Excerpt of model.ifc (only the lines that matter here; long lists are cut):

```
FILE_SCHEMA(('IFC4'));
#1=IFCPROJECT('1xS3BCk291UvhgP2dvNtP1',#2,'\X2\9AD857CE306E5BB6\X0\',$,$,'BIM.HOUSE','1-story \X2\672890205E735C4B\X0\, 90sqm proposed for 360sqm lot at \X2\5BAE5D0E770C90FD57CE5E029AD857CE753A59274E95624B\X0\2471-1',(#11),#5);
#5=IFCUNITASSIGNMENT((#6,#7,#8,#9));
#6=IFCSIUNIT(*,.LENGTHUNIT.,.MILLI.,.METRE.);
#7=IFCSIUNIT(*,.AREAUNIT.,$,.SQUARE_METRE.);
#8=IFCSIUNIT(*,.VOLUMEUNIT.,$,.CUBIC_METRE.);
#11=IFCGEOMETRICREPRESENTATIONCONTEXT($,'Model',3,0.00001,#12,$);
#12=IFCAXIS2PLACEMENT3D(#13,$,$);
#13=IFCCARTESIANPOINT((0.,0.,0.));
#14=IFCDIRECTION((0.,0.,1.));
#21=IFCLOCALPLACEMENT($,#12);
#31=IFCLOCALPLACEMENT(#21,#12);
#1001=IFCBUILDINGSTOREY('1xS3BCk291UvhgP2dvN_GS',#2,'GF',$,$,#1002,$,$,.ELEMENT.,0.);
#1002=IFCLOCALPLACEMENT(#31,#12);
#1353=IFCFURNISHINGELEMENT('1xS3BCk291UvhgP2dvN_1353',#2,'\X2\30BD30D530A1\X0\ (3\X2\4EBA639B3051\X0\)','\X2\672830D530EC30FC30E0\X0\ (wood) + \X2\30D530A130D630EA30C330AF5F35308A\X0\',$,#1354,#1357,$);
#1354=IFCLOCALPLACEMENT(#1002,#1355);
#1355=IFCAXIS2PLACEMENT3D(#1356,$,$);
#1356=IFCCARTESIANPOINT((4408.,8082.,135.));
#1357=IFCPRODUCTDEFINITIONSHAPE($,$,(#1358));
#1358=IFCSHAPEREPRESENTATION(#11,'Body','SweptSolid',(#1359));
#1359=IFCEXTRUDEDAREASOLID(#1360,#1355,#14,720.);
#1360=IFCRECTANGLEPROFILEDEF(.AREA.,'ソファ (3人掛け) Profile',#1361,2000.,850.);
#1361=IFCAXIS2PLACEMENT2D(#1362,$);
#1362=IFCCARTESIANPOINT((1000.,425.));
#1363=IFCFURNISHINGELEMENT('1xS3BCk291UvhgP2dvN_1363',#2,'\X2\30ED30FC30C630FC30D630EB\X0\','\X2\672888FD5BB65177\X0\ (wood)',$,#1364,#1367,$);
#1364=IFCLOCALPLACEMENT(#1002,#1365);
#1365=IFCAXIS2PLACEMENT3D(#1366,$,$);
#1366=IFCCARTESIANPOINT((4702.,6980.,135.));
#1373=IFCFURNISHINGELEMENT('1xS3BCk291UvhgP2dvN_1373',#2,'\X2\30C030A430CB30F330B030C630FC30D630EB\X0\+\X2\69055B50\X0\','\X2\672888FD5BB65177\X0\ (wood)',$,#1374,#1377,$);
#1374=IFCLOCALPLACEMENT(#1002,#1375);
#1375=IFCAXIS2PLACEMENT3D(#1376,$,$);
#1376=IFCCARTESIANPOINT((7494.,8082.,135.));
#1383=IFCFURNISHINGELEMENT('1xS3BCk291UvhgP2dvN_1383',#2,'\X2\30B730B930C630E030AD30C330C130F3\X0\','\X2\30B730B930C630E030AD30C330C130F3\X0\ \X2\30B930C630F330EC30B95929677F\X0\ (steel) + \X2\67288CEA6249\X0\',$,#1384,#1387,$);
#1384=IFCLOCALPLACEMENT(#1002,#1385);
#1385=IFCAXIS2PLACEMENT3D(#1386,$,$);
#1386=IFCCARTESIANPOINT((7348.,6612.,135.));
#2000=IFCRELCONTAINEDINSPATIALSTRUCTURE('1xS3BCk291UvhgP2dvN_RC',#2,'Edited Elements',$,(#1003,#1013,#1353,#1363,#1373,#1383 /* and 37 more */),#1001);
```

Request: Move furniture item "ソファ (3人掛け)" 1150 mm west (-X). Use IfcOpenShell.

```python
import ifcopenshell
import ifcopenshell.api.geometry
import ifcopenshell.util.placement

model = ifcopenshell.open("model.ifc")

item = model.by_guid("1xS3BCk291UvhgP2dvN_1353")
matrix = ifcopenshell.util.placement.get_local_placement(item.ObjectPlacement)
matrix[0, 3] -= 1150.0
ifcopenshell.api.geometry.edit_object_placement(model, product=item, matrix=matrix, is_si=False)

print(ifcopenshell.util.placement.get_local_placement(item.ObjectPlacement).round(3) + 0.0)

model.write("model-out.ifc")
```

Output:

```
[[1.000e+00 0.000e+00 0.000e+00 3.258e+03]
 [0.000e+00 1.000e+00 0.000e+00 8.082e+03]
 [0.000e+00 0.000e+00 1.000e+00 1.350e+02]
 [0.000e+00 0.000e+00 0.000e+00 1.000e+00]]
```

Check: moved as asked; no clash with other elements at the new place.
